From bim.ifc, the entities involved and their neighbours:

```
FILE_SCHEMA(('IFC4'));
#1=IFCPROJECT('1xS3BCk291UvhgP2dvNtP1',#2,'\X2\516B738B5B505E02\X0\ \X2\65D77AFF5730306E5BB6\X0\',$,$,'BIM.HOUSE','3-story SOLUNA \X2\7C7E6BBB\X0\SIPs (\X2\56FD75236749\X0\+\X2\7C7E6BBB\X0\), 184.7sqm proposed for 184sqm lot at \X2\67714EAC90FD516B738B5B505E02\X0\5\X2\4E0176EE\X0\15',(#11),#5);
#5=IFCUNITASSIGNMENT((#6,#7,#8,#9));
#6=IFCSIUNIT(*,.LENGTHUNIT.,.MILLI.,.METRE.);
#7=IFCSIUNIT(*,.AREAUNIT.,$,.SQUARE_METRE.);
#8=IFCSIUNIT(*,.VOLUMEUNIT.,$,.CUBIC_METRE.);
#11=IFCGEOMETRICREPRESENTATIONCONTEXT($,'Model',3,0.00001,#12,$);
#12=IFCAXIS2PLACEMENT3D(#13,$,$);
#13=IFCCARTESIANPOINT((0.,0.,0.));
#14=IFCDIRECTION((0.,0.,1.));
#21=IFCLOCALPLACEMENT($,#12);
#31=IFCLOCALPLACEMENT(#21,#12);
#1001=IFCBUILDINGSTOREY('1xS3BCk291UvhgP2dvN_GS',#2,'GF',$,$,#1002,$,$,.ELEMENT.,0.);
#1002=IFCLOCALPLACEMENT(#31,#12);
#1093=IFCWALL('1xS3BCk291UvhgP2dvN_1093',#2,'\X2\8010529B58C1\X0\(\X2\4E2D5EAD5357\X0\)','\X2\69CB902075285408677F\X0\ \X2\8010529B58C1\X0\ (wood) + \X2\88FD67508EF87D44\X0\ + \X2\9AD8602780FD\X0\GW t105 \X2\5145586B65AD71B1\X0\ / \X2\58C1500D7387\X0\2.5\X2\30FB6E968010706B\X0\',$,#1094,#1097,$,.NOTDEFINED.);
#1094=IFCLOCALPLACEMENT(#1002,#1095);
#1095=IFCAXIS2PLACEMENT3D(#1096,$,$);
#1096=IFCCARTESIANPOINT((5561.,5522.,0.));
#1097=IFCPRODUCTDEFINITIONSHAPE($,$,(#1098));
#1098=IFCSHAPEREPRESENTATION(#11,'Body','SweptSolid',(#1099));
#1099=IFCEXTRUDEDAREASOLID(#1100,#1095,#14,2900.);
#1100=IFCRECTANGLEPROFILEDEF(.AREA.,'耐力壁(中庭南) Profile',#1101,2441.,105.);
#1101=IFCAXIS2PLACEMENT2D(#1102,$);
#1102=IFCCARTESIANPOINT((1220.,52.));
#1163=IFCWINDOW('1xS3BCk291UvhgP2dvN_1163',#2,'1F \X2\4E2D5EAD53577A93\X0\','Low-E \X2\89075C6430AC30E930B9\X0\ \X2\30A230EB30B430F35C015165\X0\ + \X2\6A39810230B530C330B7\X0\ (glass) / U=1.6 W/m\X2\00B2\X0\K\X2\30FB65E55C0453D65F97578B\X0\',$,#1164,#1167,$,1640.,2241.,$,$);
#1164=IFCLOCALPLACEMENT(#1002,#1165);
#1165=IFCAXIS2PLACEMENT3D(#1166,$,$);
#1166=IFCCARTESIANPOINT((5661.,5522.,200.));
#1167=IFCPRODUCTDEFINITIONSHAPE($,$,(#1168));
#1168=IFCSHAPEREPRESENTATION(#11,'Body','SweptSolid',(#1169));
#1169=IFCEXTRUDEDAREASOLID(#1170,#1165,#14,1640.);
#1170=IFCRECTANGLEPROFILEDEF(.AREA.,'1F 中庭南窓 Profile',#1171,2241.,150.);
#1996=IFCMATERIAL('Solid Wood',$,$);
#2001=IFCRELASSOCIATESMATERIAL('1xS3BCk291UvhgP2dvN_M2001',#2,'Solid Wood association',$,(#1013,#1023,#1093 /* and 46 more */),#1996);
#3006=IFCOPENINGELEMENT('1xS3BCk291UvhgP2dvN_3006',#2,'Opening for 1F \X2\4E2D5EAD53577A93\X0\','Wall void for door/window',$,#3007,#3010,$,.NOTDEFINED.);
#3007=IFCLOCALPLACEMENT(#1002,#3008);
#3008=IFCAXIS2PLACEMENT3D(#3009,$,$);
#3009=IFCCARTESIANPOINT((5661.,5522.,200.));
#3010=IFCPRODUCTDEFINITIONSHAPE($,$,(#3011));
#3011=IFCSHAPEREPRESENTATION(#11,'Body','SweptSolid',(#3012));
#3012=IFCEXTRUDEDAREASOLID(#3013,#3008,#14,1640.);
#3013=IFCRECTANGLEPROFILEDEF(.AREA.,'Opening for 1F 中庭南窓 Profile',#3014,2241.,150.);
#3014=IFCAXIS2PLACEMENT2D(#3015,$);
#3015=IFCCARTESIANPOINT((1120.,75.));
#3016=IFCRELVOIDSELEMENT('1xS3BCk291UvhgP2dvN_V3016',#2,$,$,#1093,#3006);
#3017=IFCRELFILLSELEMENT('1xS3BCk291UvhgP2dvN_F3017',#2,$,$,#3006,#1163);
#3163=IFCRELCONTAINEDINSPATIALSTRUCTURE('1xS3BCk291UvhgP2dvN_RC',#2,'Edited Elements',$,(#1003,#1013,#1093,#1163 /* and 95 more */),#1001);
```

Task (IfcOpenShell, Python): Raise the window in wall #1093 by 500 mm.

```python
import numpy as np
import ifcopenshell
import ifcopenshell.api.geometry
import ifcopenshell.util.placement
import ifcopenshell.util.unit

model = ifcopenshell.open("bim.ifc")
unit_scale = ifcopenshell.util.unit.calculate_unit_scale(model)

window = model.by_guid("1xS3BCk291UvhgP2dvN_1163")
opening = window.FillsVoids[0].RelatingOpeningElement
dz = 0.5 / unit_scale

shift = np.array([0.0, 0.0, dz])
# The window is not placed relative to its opening, so move both.
for product in (opening, window):
    matrix = ifcopenshell.util.placement.get_local_placement(product.ObjectPlacement)
    matrix[:3, 3] += shift
    ifcopenshell.api.geometry.edit_object_placement(model, product=product, matrix=matrix, is_si=False)

print(f"moved by {dz * unit_scale:+.3f} m")

model.write("bim_edited.ifc")
```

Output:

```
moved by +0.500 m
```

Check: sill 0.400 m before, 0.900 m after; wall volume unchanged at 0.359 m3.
